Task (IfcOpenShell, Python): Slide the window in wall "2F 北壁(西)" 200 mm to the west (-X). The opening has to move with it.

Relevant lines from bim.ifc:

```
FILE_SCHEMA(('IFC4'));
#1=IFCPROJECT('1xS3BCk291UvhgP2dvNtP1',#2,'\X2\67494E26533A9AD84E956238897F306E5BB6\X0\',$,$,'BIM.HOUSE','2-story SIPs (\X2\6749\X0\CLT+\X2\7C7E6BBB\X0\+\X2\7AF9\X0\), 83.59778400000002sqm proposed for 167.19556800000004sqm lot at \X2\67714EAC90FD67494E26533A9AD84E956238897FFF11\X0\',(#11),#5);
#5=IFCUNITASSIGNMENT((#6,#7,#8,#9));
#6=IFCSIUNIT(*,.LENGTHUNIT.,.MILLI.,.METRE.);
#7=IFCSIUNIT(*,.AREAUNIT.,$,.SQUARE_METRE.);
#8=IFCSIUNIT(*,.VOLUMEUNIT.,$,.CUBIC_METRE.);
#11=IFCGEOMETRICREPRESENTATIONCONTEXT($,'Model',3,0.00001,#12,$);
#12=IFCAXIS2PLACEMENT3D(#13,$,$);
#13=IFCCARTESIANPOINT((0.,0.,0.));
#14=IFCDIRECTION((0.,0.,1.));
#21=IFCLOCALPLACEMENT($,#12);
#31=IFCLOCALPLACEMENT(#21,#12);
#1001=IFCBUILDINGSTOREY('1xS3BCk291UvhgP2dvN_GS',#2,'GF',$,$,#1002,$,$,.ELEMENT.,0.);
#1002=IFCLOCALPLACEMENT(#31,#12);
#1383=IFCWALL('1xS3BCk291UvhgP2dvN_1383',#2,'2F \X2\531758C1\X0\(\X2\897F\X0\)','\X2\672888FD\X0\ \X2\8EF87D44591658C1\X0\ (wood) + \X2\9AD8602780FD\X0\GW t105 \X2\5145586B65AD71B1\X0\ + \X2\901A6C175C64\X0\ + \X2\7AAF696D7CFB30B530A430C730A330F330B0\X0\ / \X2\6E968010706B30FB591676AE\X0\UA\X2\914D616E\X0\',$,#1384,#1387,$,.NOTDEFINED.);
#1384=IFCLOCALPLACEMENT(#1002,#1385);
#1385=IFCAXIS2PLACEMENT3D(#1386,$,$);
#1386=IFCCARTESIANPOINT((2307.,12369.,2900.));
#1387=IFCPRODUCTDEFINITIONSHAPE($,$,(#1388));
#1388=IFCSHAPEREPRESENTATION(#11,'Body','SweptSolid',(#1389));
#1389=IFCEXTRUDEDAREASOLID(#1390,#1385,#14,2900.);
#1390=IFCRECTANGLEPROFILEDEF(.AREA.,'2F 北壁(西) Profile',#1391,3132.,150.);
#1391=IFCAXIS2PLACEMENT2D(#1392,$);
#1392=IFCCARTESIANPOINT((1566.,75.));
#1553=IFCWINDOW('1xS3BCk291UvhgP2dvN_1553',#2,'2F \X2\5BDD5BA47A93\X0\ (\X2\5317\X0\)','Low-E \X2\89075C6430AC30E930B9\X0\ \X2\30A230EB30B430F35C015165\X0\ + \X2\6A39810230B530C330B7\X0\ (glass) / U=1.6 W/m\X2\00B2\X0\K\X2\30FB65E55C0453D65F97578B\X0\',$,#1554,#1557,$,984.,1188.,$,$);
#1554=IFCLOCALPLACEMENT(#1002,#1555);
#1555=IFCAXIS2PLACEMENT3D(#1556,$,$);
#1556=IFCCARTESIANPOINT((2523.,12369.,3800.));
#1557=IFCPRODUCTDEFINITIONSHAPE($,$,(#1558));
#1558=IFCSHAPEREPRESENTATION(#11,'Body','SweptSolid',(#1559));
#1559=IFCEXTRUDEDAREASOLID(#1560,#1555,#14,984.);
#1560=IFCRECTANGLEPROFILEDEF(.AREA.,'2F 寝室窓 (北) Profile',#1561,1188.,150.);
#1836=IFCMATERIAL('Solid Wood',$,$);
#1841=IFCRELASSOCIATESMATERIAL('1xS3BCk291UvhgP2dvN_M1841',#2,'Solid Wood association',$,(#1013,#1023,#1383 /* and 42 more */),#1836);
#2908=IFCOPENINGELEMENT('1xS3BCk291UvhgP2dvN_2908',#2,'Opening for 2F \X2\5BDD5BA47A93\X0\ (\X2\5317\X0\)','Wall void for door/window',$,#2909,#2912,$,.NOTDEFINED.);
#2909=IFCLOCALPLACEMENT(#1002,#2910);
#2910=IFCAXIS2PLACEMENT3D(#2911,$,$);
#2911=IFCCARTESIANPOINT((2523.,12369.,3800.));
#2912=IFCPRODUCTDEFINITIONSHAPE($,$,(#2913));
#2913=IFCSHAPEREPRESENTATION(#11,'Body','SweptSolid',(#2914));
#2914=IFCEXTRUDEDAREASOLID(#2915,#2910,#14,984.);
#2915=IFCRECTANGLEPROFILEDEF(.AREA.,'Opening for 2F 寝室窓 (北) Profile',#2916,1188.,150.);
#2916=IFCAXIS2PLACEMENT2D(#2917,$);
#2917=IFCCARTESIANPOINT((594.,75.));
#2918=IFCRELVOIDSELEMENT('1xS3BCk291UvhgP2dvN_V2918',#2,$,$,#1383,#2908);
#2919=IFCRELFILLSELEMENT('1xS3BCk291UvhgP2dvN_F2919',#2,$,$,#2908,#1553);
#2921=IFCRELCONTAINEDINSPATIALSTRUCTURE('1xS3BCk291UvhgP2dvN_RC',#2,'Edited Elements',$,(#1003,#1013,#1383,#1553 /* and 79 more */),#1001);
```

```python
import ifcopenshell
import ifcopenshell.api.geometry
import ifcopenshell.util.placement

model = ifcopenshell.open("bim.ifc")

window = model.by_id(1553)
opening = window.FillsVoids[0].RelatingOpeningElement
wall = opening.VoidsElements[0].RelatingBuildingElement

wall_matrix = ifcopenshell.util.placement.get_local_placement(wall.ObjectPlacement)
shift = wall_matrix[:3, 0] * -200.0
before = ifcopenshell.util.placement.get_local_placement(window.ObjectPlacement)[:3, 3].copy()

# The window is not placed relative to its opening, so move both.
for product in (opening, window):
    matrix = ifcopenshell.util.placement.get_local_placement(product.ObjectPlacement)
    matrix[:3, 3] += shift
    ifcopenshell.api.geometry.edit_object_placement(model, product=product, matrix=matrix, is_si=False)

after = ifcopenshell.util.placement.get_local_placement(window.ObjectPlacement)[:3, 3]
print("window moved by", (after - before).round(3) + 0.0)

model.write("bim-out.ifc")
```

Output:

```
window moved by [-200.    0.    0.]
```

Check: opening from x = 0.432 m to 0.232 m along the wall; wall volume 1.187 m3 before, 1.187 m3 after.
